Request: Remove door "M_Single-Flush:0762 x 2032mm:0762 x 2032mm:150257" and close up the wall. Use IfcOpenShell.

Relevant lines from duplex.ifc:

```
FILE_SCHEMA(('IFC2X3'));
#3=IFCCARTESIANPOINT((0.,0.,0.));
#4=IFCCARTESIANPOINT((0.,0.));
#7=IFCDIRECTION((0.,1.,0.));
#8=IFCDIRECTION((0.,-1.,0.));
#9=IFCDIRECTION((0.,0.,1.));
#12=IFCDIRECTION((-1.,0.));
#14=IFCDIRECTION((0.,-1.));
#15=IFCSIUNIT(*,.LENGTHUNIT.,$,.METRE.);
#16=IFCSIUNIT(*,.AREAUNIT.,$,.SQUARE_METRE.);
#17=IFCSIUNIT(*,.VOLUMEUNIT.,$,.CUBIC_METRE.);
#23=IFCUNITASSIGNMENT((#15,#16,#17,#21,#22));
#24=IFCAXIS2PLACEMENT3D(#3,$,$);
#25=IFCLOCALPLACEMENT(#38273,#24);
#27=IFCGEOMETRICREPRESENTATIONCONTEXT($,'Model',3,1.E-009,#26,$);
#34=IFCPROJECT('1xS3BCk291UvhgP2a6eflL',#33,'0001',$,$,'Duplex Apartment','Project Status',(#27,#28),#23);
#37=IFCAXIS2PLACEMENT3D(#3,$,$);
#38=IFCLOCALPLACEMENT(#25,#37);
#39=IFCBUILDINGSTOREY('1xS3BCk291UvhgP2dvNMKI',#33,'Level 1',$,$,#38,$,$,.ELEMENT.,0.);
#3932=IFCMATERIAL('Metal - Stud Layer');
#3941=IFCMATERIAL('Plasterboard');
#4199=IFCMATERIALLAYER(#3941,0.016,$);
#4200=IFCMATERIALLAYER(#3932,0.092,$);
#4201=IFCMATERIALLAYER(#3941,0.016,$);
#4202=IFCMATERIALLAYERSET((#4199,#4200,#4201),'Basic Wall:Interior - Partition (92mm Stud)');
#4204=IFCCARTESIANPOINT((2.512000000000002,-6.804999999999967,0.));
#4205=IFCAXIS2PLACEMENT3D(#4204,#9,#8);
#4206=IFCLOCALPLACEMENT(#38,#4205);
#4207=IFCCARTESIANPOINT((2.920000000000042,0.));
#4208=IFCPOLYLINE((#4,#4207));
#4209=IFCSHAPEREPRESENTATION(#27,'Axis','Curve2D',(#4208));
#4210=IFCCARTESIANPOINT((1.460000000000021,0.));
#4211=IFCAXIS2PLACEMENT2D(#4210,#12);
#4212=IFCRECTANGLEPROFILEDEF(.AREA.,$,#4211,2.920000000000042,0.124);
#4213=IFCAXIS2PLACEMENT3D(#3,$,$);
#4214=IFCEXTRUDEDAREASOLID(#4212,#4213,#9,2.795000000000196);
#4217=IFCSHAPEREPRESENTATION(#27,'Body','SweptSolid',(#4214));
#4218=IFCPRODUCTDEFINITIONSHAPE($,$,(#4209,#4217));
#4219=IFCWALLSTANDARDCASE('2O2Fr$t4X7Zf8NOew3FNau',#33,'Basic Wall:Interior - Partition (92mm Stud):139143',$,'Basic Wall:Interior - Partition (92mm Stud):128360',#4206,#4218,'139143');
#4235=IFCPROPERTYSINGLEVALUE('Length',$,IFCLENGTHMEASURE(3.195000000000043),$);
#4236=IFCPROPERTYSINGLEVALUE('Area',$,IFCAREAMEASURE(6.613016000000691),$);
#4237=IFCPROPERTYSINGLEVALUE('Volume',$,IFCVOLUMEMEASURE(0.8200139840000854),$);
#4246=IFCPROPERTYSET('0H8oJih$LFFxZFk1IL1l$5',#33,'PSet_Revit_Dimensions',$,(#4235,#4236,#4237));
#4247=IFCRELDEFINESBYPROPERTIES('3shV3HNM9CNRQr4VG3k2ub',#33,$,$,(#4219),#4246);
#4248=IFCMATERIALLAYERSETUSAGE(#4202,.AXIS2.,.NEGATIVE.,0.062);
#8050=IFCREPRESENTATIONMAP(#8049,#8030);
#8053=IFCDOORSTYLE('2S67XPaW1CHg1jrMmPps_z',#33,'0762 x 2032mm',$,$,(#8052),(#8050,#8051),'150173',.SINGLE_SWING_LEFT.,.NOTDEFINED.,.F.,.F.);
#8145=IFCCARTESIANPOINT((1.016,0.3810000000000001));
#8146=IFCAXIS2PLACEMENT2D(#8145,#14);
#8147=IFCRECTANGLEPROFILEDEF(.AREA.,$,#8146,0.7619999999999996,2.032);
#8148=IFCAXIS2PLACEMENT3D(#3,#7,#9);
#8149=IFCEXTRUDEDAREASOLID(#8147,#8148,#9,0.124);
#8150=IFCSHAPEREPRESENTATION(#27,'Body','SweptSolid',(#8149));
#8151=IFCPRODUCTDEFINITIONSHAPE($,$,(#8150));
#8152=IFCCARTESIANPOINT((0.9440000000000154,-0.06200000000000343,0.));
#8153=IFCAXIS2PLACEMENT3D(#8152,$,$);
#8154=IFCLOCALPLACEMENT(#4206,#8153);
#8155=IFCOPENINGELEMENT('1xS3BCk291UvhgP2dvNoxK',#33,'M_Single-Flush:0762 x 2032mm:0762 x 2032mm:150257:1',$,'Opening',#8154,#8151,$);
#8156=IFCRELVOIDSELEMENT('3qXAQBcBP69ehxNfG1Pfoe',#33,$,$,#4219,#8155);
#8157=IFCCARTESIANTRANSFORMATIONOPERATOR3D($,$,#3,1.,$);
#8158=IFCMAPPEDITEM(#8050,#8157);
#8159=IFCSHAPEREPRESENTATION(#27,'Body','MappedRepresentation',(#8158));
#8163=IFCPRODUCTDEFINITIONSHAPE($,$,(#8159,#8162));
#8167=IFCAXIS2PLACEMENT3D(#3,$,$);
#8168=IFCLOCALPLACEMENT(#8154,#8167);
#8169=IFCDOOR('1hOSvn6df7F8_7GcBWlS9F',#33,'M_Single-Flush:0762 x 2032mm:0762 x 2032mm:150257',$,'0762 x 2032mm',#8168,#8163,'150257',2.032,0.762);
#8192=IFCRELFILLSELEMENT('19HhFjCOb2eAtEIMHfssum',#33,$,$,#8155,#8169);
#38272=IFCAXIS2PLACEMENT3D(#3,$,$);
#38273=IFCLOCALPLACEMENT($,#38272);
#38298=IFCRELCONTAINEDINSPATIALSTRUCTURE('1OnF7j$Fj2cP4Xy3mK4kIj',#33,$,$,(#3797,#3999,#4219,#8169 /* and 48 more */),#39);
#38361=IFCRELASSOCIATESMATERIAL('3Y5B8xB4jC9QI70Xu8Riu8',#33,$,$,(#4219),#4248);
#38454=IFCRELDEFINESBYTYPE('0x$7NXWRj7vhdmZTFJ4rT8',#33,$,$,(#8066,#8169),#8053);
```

```python
import ifcopenshell
import ifcopenshell.api.feature
import ifcopenshell.api.pset
import ifcopenshell.api.root
import ifcopenshell.geom
import ifcopenshell.util.element
import ifcopenshell.util.shape
import ifcopenshell.util.unit

model = ifcopenshell.open("duplex.ifc")
area_scale = ifcopenshell.util.unit.calculate_unit_scale(model, "AREAUNIT")
volume_scale = ifcopenshell.util.unit.calculate_unit_scale(model, "VOLUMEUNIT")
settings = ifcopenshell.geom.settings()


def volume(element):
    """Net volume in cubic metres, openings subtracted."""
    shape = ifcopenshell.geom.create_shape(settings, element)
    return ifcopenshell.util.shape.get_volume(shape.geometry)


door = model.by_guid("1hOSvn6df7F8_7GcBWlS9F")
opening = door.FillsVoids[0].RelatingOpeningElement
wall = opening.VoidsElements[0].RelatingBuildingElement
before = volume(wall)

ifcopenshell.api.root.remove_product(model, product=door)
ifcopenshell.api.feature.remove_feature(model, feature=opening)

after = volume(wall)
thickness = 0.124  # wall thickness in metres

# Update the wall's stored quantities.
pset = model.by_id(ifcopenshell.util.element.get_pset(wall, "PSet_Revit_Dimensions", should_inherit=False)["id"])
ifcopenshell.api.pset.edit_pset(model, pset=pset, properties={
    "Area": model.create_entity("IfcAreaMeasure", after / thickness / area_scale),
    "Volume": model.create_entity("IfcVolumeMeasure", after / volume_scale),
})

print(f"wall volume {before:.3f} -> {after:.3f} m3")

model.write("duplex-out.ifc")
```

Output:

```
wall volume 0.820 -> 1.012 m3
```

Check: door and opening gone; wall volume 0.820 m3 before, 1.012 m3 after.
